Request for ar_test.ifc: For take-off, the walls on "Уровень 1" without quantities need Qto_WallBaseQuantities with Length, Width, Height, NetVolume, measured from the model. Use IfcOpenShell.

First a look at what the model holds.

```python
import ifcopenshell
import ifcopenshell.util.element
import ifcopenshell.util.unit

model = ifcopenshell.open("ar_test.ifc")
print(model.schema)
for unit_type in ("LENGTHUNIT", "AREAUNIT", "VOLUMEUNIT"):
    print(unit_type, ifcopenshell.util.unit.calculate_unit_scale(model, unit_type))
storey = next(s for s in model.by_type("IfcBuildingStorey") if s.Name == "Уровень 1")
walls = [e for e in ifcopenshell.util.element.get_decomposition(storey) if e.is_a("IfcWall")]
for e in sorted(walls, key=lambda e: e.id()):
    print(e.id(), e.is_a(), e.Name, list(ifcopenshell.util.element.get_psets(e, qtos_only=True)), sep=" | ")
```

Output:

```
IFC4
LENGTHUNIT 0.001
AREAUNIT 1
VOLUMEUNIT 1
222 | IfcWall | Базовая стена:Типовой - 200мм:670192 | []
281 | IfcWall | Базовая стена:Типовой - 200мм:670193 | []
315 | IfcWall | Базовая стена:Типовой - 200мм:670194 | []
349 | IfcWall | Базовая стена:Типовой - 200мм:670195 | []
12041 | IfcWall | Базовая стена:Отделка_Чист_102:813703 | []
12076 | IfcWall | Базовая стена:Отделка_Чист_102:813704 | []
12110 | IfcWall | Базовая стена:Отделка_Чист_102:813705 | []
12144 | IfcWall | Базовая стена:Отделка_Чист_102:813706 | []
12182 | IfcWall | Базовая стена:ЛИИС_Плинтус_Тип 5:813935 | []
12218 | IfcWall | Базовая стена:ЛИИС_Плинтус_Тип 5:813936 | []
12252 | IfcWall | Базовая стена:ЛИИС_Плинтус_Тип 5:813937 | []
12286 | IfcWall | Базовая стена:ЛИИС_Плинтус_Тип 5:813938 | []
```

```python
import ifcopenshell
import ifcopenshell.api.pset
import ifcopenshell.geom
import ifcopenshell.util.element
import ifcopenshell.util.shape
import ifcopenshell.util.unit

model = ifcopenshell.open("ar_test.ifc")
unit_scale = ifcopenshell.util.unit.calculate_unit_scale(model)
volume_scale = ifcopenshell.util.unit.calculate_unit_scale(model, "VOLUMEUNIT")
settings = ifcopenshell.geom.settings()

storey = next(s for s in model.by_type("IfcBuildingStorey") if s.Name == "Уровень 1")
walls = [e for e in ifcopenshell.util.element.get_decomposition(storey) if e.is_a("IfcWall")]

for e in sorted(walls, key=lambda e: e.id()):
    if ifcopenshell.util.element.get_psets(e, qtos_only=True, should_inherit=False):
        continue
    # Geometry comes back in metres, in the element's own axes.
    shape = ifcopenshell.geom.create_shape(settings, e)
    values = {
        "Length": ifcopenshell.util.shape.get_x(shape.geometry) / unit_scale,
        "Width": ifcopenshell.util.shape.get_y(shape.geometry) / unit_scale,
        "Height": ifcopenshell.util.shape.get_z(shape.geometry) / unit_scale,
        "NetVolume": ifcopenshell.util.shape.get_volume(shape.geometry) / volume_scale,
    }
    qto = ifcopenshell.api.pset.add_qto(model, product=e, name="Qto_WallBaseQuantities")
    ifcopenshell.api.pset.edit_qto(model, qto=qto, properties=values)
    print(e.id(), {k: round(v, 3) for k, v in values.items()})

model.write("ar_test_rev.ifc")
```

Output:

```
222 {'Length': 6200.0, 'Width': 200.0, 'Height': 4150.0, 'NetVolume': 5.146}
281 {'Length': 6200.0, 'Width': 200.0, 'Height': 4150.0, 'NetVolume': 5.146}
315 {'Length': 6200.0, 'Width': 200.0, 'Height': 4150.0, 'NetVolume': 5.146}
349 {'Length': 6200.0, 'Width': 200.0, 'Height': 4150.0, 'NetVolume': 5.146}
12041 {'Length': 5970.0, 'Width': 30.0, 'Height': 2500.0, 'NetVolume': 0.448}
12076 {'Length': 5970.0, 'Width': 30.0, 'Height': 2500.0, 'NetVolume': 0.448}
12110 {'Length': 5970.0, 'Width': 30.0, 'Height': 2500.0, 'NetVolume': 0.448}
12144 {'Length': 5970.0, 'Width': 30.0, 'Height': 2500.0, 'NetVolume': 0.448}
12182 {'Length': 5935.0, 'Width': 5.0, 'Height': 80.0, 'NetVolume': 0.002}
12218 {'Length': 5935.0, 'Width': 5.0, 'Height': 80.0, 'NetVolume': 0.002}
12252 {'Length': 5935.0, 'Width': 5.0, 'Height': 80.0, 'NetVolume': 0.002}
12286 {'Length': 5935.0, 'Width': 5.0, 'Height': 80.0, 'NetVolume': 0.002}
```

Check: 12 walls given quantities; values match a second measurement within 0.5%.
